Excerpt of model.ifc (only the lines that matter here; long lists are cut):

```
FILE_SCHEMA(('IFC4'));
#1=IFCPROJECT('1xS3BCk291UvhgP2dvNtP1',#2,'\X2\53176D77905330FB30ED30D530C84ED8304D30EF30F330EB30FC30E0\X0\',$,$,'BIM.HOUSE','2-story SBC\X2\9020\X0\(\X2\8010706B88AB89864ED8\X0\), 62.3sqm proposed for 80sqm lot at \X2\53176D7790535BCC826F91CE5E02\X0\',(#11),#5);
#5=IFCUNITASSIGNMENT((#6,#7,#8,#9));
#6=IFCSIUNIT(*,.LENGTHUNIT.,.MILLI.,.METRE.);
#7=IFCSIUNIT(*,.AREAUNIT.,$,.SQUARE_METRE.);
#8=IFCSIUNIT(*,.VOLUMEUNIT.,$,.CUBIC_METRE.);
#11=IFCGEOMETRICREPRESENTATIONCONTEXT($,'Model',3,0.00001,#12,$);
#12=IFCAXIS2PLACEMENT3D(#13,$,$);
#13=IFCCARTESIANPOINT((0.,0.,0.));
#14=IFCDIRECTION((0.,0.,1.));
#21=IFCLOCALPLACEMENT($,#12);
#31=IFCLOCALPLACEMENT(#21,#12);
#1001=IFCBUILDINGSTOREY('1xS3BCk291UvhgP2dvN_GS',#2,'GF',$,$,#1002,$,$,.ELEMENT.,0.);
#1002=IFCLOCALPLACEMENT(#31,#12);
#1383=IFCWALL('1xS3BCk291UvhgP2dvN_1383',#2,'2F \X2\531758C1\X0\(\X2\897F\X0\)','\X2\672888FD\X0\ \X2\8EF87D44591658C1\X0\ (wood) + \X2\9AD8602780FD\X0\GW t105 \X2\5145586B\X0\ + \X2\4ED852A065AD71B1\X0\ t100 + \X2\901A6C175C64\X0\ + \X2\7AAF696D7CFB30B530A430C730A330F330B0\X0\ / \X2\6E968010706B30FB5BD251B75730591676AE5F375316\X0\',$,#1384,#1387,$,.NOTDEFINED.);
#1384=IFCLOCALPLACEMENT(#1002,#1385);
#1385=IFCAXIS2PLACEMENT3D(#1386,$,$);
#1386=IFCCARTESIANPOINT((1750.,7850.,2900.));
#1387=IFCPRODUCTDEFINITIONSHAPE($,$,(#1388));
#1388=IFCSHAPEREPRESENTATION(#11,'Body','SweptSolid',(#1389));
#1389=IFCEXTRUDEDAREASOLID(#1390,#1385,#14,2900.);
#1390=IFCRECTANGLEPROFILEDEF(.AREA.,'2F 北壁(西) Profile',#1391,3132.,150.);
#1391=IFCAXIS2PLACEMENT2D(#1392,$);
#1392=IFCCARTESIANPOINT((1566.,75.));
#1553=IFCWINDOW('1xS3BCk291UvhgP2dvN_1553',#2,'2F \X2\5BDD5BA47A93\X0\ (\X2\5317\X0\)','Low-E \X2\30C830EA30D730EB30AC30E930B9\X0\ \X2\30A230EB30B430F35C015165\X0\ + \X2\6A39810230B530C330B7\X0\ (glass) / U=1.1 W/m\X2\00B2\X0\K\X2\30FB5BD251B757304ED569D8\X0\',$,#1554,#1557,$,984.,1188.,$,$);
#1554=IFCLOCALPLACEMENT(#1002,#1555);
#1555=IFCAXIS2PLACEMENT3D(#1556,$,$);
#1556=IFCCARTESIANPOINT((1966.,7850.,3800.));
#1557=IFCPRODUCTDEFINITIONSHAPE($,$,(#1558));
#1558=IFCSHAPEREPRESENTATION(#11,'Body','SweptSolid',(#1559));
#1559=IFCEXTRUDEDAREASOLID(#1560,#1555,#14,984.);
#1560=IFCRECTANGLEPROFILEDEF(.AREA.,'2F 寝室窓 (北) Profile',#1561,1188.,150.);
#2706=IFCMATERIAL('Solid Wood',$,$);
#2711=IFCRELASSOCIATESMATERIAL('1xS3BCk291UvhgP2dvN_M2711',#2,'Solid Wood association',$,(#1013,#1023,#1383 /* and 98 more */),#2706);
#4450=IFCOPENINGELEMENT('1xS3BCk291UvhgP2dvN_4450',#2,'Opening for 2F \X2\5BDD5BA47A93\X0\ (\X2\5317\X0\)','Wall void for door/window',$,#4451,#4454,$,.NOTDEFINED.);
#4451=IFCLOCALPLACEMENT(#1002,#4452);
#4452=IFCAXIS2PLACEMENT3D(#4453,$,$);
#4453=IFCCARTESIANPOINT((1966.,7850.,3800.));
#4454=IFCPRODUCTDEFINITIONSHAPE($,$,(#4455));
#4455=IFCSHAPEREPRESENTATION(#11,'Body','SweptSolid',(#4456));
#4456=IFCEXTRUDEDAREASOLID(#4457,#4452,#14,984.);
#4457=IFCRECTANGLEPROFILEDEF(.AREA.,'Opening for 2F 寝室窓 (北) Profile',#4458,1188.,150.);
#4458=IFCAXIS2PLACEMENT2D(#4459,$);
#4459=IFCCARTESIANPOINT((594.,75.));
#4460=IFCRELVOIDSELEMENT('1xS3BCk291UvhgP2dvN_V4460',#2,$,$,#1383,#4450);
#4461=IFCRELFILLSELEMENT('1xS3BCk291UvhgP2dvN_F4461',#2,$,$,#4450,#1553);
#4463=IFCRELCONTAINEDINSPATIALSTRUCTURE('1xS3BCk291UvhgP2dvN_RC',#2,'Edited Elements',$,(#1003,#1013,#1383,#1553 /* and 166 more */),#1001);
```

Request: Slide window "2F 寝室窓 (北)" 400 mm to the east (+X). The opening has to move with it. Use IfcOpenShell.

```python
import ifcopenshell
import ifcopenshell.api.geometry
import ifcopenshell.util.placement

model = ifcopenshell.open("model.ifc")

window = model.by_id(1553)
opening = window.FillsVoids[0].RelatingOpeningElement
wall = opening.VoidsElements[0].RelatingBuildingElement

wall_matrix = ifcopenshell.util.placement.get_local_placement(wall.ObjectPlacement)
shift = wall_matrix[:3, 0] * 400.0
before = ifcopenshell.util.placement.get_local_placement(window.ObjectPlacement)[:3, 3].copy()

# The window is not placed relative to its opening, so move both.
for product in (opening, window):
    matrix = ifcopenshell.util.placement.get_local_placement(product.ObjectPlacement)
    matrix[:3, 3] += shift
    ifcopenshell.api.geometry.edit_object_placement(model, product=product, matrix=matrix, is_si=False)

after = ifcopenshell.util.placement.get_local_placement(window.ObjectPlacement)[:3, 3]
print("window moved by", (after - before).round(3) + 0.0)

model.write("model_edited.ifc")
```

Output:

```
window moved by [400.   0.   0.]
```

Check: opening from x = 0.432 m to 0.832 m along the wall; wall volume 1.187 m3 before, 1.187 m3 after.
